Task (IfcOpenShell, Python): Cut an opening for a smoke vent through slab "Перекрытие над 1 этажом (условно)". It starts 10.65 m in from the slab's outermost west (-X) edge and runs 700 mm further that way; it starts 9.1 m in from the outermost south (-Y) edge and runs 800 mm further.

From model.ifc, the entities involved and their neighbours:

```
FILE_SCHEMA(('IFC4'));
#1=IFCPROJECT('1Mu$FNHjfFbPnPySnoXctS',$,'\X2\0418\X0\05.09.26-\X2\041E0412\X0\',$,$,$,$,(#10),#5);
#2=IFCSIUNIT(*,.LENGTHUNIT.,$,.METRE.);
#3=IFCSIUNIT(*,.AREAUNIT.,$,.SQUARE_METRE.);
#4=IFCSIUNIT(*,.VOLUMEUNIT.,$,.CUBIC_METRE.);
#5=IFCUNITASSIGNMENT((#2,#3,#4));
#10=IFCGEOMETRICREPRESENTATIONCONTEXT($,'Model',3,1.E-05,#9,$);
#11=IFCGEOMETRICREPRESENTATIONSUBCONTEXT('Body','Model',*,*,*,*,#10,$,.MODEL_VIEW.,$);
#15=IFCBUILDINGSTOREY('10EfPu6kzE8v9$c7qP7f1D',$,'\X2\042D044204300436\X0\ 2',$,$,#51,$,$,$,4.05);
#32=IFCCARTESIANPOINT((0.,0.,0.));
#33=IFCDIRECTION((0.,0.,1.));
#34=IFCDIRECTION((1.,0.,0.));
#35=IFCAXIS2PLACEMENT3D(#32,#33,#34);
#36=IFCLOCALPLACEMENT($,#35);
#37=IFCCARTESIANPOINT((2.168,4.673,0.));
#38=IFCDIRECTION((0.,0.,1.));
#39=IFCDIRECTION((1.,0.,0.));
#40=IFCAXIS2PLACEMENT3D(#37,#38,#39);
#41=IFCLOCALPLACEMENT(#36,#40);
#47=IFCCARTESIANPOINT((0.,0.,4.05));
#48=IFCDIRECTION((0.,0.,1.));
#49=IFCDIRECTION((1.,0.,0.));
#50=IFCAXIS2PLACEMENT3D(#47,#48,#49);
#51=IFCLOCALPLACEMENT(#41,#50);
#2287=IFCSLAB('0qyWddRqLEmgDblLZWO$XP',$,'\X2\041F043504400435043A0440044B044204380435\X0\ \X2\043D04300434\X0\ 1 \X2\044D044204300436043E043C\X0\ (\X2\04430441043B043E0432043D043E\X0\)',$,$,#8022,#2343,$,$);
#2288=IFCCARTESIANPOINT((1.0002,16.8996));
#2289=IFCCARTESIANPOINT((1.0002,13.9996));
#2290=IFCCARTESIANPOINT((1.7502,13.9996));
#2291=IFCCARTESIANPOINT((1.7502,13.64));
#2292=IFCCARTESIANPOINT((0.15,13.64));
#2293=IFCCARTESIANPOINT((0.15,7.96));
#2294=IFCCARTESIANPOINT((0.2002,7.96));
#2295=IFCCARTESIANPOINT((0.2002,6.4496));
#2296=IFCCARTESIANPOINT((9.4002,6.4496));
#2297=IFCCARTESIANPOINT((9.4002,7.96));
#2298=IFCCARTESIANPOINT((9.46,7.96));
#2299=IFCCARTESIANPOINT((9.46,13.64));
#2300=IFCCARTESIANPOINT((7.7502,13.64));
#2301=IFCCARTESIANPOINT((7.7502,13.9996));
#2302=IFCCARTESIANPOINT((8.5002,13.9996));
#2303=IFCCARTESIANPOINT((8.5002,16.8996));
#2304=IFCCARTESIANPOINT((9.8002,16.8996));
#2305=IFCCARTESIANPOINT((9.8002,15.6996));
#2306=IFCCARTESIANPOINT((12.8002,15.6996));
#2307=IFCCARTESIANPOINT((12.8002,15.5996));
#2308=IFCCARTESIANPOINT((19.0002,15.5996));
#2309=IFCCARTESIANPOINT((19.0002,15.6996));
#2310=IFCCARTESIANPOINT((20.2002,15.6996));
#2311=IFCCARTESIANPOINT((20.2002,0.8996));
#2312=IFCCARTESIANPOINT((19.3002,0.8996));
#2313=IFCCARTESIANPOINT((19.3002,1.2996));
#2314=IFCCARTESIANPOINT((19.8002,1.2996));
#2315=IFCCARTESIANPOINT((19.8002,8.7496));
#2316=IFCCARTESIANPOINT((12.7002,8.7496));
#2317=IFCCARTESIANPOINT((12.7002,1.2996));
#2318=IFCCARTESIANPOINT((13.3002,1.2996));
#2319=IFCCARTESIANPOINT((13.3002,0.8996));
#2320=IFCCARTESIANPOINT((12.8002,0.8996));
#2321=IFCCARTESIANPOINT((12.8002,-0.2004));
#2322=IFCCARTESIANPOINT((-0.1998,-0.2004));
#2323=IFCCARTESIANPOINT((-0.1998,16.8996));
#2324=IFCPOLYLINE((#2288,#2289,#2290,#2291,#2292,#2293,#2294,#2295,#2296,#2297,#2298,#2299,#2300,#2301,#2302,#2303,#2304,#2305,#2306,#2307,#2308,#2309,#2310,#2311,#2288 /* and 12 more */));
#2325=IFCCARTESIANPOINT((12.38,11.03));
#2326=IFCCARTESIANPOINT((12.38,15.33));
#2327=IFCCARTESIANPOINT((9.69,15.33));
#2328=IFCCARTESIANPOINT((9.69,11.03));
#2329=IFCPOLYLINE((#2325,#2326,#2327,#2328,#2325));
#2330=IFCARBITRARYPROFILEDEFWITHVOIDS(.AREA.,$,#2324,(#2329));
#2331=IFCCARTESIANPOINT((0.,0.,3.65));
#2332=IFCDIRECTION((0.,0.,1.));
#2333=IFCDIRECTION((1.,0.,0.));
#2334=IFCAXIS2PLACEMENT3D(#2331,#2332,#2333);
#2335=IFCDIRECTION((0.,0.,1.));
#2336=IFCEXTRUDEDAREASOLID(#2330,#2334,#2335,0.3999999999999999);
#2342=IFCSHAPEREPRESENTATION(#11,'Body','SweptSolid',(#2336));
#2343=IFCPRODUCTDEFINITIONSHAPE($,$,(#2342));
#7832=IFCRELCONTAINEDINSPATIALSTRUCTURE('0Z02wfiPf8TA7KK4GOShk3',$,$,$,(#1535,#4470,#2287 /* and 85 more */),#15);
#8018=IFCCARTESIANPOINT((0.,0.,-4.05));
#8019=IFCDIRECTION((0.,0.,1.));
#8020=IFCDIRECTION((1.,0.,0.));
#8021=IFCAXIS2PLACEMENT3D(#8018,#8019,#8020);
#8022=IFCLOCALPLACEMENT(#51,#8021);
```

```python
import numpy as np
import ifcopenshell
import ifcopenshell.api.feature
import ifcopenshell.api.geometry
import ifcopenshell.api.root
import ifcopenshell.geom
import ifcopenshell.util.placement
import ifcopenshell.util.representation
import ifcopenshell.util.shape
import ifcopenshell.util.unit

model = ifcopenshell.open("model.ifc")
unit_scale = ifcopenshell.util.unit.calculate_unit_scale(model)
settings = ifcopenshell.geom.settings()


def volume(element):
    """Net volume in cubic metres, openings subtracted."""
    shape = ifcopenshell.geom.create_shape(settings, element)
    return ifcopenshell.util.shape.get_volume(shape.geometry)


slab = model.by_guid("0qyWddRqLEmgDblLZWO$XP")
before = volume(slab)

# Extent in the slab's own axes, in metres. The edges named are its -X and -Y sides.
slab_shape = ifcopenshell.geom.create_shape(settings, slab)
vertices = ifcopenshell.util.shape.get_vertices(slab_shape.geometry)
x_min, y_min, bottom = vertices.min(axis=0)
top = vertices[:, 2].max()

opening = ifcopenshell.api.root.create_entity(model, ifc_class="IfcOpeningElement", name="Smoke vent opening", predefined_type="OPENING")
context = ifcopenshell.util.representation.get_context(model, "Model", "Body", "MODEL_VIEW")
width, depth = 0.7, 0.8
outline = [(0.0, 0.0), (width, 0.0), (width, depth), (0.0, depth), (0.0, 0.0)]
# Overshoot both faces by 50 mm so the cut is clean.
shape = ifcopenshell.api.geometry.add_slab_representation(
    model, context=context, depth=top - bottom + 0.1, polyline=outline
)
ifcopenshell.api.geometry.assign_representation(model, product=opening, representation=shape)

matrix = ifcopenshell.util.placement.get_local_placement(slab.ObjectPlacement)
matrix[:, 3] = matrix @ np.append(np.array([x_min + 10.65, y_min + 9.1, bottom - 0.05]) / unit_scale, 1.0)
ifcopenshell.api.geometry.edit_object_placement(model, product=opening, matrix=matrix, is_si=False)
ifcopenshell.api.feature.add_feature(model, feature=opening, element=slab)

after = volume(slab)

print(f"slab volume {before:.3f} -> {after:.3f} m3")

model.write("model_v2.ifc")
```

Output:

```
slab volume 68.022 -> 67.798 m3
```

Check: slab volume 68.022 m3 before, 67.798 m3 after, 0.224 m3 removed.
